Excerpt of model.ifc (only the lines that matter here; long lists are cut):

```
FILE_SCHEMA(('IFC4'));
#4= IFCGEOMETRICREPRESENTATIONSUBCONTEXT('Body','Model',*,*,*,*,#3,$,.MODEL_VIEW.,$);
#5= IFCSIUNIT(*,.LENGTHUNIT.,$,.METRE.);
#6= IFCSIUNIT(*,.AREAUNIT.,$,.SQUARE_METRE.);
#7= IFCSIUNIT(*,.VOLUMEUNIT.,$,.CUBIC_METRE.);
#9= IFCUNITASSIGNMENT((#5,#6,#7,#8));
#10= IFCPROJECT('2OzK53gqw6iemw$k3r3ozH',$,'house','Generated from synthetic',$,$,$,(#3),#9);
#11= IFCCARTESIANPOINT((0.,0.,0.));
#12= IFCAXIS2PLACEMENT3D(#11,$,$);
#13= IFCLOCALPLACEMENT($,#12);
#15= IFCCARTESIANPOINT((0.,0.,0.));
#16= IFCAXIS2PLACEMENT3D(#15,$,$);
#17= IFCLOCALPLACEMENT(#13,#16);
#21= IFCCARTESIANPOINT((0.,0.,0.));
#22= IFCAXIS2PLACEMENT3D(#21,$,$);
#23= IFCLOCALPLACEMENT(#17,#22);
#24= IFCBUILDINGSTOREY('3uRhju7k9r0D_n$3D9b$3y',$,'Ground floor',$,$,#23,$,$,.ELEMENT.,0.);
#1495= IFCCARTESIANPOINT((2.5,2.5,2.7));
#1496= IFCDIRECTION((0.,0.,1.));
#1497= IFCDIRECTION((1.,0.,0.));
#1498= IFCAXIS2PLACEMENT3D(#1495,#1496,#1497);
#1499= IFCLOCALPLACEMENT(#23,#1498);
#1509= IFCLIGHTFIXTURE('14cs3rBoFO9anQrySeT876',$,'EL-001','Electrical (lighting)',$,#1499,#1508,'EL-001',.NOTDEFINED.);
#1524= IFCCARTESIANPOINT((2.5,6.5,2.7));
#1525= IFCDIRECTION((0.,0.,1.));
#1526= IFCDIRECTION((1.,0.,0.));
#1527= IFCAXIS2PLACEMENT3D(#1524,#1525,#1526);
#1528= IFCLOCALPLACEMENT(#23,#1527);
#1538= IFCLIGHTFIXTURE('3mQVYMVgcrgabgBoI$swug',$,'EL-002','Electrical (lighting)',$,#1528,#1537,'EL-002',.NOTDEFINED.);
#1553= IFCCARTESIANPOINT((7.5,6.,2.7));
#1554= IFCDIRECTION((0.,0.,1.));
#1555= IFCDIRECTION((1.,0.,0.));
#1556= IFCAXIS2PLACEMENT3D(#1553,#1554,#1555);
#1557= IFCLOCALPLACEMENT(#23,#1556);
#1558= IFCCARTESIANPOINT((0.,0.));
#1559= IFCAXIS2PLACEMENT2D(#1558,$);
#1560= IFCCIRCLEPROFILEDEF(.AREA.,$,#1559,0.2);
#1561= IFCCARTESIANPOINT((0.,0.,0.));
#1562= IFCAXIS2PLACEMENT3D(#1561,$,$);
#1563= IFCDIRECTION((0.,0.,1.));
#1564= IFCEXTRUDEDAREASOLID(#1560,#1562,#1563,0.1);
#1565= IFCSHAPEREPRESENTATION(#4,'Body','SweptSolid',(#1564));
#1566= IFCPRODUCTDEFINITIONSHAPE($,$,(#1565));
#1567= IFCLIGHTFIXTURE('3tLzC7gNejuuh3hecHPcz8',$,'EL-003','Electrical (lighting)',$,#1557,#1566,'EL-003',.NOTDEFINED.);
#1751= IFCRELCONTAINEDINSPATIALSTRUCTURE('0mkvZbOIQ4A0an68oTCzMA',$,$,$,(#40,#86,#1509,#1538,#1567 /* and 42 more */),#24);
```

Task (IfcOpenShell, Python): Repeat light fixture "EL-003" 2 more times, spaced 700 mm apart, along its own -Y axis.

```python
import ifcopenshell
import ifcopenshell.api.geometry
import ifcopenshell.api.root
import ifcopenshell.util.element
import ifcopenshell.util.placement
import ifcopenshell.util.unit

model = ifcopenshell.open("model.ifc")
unit_scale = ifcopenshell.util.unit.calculate_unit_scale(model)

source = model.by_guid("3tLzC7gNejuuh3hecHPcz8")
base = ifcopenshell.util.placement.get_local_placement(source.ObjectPlacement)
step = -base[:3, 1] * 0.7 / unit_scale

for i in range(1, 3):
    copy = ifcopenshell.api.root.copy_class(model, product=source)
    copy.Representation = ifcopenshell.util.element.copy_deep(
        model, source.Representation, exclude=["IfcGeometricRepresentationContext", "IfcRepresentationMap"]
    )
    copy.Tag = None
    matrix = base.copy()
    matrix[:3, 3] += i * step
    print("added at", matrix[:3, 3].round(3) + 0.0)
    ifcopenshell.api.geometry.edit_object_placement(model, product=copy, matrix=matrix, is_si=False)

model.write("model_rev.ifc")
```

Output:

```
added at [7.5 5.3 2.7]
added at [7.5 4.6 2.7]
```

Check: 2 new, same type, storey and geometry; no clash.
